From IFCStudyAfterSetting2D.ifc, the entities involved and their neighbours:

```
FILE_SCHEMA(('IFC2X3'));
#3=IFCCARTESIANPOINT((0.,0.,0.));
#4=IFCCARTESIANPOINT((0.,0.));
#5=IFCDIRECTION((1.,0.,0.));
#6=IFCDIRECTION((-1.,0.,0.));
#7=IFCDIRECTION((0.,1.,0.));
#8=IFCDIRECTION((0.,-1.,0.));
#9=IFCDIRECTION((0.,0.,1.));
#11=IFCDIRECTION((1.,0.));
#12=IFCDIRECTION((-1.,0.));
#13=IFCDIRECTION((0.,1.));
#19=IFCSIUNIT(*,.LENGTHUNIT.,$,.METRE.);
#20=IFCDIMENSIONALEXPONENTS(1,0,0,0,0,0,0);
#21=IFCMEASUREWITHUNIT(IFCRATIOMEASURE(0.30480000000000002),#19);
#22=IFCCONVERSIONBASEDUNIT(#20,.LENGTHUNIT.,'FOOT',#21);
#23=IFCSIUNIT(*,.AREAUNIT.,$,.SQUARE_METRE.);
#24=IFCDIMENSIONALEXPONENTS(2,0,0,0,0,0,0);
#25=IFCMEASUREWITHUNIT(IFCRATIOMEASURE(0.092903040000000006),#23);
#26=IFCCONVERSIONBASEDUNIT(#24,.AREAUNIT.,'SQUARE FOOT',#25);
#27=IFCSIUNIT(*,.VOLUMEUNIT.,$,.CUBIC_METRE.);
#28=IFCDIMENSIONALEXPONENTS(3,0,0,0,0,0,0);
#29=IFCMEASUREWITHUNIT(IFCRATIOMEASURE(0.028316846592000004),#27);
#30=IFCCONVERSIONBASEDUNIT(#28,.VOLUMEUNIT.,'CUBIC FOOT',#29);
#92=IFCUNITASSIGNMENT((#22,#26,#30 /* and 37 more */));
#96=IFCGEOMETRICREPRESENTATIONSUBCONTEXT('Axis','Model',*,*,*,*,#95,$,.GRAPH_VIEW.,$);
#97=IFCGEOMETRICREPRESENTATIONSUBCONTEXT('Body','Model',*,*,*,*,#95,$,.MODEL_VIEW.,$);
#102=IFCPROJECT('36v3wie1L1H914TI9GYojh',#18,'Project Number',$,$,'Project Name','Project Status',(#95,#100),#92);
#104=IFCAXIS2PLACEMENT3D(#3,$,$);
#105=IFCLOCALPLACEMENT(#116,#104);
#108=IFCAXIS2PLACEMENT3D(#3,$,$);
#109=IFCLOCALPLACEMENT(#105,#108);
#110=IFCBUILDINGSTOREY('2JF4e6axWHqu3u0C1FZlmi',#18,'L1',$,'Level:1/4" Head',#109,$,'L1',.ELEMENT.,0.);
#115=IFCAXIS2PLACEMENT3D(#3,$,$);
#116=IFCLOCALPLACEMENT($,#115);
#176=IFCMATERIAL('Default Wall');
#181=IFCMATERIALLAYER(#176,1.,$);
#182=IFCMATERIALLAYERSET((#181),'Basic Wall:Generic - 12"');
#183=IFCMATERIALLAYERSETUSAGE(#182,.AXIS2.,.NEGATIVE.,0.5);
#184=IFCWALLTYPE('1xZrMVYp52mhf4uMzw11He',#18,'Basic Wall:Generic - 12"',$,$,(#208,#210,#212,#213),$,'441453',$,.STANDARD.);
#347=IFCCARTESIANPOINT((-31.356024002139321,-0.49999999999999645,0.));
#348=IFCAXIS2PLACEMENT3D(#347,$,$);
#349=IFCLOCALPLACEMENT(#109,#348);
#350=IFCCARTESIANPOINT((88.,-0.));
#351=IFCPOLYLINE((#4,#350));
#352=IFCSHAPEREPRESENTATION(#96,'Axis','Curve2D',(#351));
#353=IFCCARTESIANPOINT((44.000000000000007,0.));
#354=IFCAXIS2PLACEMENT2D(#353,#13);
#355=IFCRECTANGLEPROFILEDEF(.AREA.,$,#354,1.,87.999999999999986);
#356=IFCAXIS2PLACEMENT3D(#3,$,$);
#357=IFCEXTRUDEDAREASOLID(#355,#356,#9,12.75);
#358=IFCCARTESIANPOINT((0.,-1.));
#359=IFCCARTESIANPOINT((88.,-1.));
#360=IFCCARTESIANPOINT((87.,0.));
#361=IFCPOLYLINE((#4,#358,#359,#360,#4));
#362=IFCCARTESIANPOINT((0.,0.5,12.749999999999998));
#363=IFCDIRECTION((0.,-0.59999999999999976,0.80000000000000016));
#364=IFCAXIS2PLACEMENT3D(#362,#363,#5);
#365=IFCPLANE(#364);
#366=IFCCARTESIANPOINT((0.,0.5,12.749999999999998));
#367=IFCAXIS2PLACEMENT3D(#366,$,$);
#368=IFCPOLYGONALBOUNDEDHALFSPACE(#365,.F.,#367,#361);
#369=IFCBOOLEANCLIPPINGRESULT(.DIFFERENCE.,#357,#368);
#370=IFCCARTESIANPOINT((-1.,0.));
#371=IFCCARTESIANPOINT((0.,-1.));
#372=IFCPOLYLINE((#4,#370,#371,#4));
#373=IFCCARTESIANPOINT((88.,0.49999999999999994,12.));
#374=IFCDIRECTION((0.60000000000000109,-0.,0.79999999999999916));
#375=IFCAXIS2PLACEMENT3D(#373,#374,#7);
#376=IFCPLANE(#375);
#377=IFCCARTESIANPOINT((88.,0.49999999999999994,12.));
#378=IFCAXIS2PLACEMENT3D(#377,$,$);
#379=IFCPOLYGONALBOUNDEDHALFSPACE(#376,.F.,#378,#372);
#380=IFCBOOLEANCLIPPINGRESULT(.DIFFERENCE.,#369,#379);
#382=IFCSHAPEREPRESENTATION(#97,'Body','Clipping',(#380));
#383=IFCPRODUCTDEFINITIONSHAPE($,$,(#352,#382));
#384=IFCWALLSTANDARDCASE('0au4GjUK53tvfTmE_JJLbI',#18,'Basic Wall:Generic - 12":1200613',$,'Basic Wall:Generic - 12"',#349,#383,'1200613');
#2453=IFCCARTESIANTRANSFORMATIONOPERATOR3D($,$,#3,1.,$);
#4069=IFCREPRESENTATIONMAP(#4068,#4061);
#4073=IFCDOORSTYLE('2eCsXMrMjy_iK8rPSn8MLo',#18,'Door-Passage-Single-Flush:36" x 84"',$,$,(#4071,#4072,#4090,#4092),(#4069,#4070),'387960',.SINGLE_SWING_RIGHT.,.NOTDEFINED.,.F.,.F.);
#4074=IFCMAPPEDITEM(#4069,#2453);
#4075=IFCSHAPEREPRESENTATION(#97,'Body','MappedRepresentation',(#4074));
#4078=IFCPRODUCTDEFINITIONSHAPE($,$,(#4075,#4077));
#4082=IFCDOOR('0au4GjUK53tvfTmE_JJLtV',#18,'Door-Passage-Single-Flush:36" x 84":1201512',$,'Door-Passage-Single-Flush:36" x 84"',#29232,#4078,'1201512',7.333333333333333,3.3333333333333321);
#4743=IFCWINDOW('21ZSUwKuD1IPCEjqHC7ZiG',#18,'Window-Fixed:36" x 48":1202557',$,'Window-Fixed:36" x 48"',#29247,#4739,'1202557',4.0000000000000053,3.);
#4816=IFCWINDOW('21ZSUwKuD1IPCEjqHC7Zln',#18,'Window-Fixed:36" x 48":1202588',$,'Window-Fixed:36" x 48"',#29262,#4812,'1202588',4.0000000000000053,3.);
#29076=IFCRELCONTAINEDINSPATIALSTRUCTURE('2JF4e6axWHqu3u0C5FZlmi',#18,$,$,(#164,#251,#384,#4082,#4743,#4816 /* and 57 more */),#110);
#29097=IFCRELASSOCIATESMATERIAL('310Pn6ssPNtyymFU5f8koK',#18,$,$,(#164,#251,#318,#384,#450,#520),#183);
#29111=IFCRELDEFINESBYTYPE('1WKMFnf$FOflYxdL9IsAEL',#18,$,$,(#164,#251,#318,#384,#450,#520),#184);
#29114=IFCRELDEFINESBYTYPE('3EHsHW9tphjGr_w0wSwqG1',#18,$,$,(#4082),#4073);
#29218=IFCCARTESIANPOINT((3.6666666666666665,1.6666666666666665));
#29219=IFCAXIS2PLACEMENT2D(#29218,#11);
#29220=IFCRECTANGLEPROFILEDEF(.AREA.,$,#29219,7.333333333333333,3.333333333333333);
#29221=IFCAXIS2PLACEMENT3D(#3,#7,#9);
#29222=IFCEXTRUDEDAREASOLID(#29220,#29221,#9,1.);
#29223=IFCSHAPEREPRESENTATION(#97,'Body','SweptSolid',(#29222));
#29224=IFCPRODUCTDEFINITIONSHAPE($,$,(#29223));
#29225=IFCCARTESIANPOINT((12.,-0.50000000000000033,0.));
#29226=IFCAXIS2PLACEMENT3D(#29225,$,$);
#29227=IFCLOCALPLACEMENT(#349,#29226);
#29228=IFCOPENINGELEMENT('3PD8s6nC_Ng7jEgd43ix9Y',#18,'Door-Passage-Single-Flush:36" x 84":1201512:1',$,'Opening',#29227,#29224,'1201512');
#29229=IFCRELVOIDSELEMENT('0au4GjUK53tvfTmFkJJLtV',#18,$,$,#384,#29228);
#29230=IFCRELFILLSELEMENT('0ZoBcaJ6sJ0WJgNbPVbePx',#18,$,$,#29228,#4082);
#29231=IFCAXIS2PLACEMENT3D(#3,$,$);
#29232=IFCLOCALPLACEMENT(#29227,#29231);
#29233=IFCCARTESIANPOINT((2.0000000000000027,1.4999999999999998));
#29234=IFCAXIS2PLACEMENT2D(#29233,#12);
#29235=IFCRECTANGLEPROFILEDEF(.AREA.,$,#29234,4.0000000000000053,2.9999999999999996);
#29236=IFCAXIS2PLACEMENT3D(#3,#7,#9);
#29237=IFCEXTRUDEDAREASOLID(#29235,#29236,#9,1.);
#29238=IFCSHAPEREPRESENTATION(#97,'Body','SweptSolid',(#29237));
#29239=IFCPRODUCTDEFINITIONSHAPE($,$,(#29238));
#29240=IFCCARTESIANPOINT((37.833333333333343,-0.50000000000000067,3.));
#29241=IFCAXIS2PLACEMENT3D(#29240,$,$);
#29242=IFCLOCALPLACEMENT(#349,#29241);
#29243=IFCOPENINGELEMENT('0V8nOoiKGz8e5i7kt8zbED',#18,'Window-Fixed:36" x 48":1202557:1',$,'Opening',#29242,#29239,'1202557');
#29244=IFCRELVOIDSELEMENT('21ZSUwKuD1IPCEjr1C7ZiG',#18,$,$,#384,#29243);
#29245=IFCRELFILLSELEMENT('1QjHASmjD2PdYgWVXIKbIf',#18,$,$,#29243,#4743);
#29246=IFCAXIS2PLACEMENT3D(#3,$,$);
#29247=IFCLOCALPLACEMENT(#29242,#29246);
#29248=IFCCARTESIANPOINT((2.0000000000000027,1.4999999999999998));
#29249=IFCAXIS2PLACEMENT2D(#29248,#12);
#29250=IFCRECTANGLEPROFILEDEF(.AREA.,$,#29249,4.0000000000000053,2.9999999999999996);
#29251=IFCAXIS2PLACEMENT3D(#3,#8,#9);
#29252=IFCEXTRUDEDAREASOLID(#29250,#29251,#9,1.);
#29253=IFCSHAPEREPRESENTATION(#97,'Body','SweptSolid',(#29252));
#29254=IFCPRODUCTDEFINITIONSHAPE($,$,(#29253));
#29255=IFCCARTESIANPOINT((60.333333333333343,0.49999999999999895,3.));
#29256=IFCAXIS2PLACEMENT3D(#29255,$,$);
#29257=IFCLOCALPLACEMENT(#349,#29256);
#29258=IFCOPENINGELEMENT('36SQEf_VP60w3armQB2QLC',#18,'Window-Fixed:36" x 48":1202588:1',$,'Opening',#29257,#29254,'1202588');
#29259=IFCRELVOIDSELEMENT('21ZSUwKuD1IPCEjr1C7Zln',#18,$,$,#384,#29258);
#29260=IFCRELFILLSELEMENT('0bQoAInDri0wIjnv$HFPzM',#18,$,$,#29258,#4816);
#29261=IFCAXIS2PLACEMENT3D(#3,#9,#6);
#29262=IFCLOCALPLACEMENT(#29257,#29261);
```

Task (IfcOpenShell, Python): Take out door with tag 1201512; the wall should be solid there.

```python
import ifcopenshell
import ifcopenshell.api.feature
import ifcopenshell.api.root
import ifcopenshell.geom
import ifcopenshell.util.shape

model = ifcopenshell.open("IFCStudyAfterSetting2D.ifc")
settings = ifcopenshell.geom.settings()


def volume(element):
    """Net volume in cubic metres, openings subtracted."""
    shape = ifcopenshell.geom.create_shape(settings, element)
    return ifcopenshell.util.shape.get_volume(shape.geometry)


door = model.by_guid("0au4GjUK53tvfTmE_JJLtV")
opening = door.FillsVoids[0].RelatingOpeningElement
wall = opening.VoidsElements[0].RelatingBuildingElement
before = volume(wall)

ifcopenshell.api.root.remove_product(model, product=door)
ifcopenshell.api.feature.remove_feature(model, feature=opening)

after = volume(wall)

print(f"wall volume {before:.3f} -> {after:.3f} m3")

model.write("IFCStudyAfterSetting2D_rev.ifc")
```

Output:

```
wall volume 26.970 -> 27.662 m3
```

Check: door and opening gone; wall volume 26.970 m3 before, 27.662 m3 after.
